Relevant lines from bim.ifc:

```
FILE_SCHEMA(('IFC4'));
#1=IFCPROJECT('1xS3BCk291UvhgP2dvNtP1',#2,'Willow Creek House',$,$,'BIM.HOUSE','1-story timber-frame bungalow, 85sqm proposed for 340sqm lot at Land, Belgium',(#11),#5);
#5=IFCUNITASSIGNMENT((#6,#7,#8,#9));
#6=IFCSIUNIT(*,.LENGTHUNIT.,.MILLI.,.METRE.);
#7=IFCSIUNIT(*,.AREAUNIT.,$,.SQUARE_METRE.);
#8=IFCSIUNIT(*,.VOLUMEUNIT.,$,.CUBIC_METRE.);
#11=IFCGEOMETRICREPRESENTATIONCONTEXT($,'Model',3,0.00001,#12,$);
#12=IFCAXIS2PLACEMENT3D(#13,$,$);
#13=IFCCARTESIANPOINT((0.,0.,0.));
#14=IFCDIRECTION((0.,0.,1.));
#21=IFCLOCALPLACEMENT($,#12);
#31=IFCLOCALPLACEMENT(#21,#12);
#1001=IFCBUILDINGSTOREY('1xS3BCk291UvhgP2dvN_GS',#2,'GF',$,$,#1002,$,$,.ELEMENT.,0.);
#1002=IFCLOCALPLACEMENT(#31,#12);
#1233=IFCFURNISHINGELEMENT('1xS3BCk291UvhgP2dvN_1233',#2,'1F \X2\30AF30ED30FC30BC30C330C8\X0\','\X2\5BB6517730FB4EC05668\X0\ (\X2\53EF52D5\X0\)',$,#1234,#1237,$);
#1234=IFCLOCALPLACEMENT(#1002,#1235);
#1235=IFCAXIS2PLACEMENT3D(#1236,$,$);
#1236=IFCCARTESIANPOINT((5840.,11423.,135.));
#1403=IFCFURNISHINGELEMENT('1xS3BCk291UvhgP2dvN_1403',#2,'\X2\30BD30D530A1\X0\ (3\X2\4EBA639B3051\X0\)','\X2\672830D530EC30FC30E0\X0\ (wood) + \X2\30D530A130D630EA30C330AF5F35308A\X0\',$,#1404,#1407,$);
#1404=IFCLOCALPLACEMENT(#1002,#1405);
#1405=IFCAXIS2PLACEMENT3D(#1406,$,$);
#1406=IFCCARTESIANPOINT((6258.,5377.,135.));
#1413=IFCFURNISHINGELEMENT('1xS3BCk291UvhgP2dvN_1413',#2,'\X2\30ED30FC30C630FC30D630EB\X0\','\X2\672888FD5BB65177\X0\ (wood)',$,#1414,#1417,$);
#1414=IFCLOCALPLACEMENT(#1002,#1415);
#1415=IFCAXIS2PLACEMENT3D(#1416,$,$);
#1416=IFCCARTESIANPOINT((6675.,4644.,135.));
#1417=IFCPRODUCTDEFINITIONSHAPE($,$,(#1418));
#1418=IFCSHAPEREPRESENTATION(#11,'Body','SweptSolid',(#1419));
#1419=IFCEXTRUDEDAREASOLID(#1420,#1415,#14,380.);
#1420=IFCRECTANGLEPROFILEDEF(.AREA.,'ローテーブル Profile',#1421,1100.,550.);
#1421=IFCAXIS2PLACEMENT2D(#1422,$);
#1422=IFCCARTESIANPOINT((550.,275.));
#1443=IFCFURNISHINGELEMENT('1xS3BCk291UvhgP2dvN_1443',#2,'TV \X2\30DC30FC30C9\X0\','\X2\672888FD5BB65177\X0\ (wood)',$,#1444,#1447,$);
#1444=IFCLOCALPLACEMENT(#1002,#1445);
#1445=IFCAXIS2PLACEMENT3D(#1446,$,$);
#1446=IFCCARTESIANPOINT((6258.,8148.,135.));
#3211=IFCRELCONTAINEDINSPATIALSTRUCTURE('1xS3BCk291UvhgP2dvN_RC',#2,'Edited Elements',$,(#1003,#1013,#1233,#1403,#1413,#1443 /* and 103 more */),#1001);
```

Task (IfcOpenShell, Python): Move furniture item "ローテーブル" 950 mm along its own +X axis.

```python
import ifcopenshell
import ifcopenshell.api.geometry
import ifcopenshell.util.placement
import ifcopenshell.util.unit

model = ifcopenshell.open("bim.ifc")
unit_scale = ifcopenshell.util.unit.calculate_unit_scale(model)

item = model.by_guid("1xS3BCk291UvhgP2dvN_1413")
matrix = ifcopenshell.util.placement.get_local_placement(item.ObjectPlacement)
matrix[:3, 3] += matrix[:3, 0] * 0.95 / unit_scale
ifcopenshell.api.geometry.edit_object_placement(model, product=item, matrix=matrix, is_si=False)

print(ifcopenshell.util.placement.get_local_placement(item.ObjectPlacement).round(3) + 0.0)

model.write("bim-out.ifc")
```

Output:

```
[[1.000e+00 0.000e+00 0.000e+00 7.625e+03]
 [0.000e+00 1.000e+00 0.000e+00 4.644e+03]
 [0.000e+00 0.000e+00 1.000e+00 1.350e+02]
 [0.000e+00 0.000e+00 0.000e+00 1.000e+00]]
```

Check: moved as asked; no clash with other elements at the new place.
